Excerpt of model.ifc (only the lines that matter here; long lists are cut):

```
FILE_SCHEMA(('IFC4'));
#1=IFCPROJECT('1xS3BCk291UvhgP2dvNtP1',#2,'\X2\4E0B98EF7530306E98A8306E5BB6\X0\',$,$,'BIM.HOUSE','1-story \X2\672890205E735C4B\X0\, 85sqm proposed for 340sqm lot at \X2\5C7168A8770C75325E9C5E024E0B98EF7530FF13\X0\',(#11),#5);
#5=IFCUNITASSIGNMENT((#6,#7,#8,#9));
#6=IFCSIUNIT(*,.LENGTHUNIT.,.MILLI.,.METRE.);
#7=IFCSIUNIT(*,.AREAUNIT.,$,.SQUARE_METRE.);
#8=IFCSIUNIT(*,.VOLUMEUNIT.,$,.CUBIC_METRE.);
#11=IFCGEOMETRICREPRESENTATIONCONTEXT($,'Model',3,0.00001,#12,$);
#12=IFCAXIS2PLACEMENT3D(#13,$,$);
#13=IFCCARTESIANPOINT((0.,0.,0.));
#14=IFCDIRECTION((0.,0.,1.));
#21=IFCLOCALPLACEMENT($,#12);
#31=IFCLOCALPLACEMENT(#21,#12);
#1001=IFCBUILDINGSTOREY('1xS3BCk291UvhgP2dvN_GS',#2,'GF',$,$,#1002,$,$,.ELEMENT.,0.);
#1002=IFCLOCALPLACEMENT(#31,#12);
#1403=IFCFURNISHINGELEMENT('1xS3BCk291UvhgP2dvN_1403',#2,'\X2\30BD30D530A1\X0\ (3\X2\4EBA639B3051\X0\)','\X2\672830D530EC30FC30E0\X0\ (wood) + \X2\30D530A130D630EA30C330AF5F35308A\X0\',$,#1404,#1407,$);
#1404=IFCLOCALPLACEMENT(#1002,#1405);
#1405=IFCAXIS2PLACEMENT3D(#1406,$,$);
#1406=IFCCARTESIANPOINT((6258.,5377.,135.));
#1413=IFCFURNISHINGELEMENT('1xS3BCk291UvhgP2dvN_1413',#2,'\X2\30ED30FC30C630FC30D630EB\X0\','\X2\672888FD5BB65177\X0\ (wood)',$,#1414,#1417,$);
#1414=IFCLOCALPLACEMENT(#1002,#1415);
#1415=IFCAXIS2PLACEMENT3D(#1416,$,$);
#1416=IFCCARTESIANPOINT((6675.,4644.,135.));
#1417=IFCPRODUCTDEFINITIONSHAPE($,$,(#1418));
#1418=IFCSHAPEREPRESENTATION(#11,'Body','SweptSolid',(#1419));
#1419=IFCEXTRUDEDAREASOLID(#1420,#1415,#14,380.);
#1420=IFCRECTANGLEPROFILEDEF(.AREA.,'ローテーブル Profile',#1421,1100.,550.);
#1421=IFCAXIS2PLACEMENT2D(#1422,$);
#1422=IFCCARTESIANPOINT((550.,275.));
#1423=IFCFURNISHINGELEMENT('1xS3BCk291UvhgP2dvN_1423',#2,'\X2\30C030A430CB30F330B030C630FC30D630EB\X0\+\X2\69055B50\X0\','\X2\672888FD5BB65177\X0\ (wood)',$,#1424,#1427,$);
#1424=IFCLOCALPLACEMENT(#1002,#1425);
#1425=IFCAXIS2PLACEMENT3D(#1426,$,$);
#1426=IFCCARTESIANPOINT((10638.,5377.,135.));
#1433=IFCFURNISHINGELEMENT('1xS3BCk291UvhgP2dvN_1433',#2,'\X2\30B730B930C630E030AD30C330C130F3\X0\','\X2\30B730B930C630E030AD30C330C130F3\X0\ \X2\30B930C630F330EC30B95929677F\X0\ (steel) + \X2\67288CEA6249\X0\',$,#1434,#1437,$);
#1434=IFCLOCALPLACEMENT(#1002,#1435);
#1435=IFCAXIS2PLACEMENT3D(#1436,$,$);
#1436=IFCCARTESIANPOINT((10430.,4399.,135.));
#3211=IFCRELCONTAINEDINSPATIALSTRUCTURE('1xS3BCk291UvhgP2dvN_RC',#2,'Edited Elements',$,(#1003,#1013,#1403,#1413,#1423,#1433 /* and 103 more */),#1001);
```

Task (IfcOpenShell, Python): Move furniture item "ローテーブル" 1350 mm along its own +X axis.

```python
import ifcopenshell
import ifcopenshell.api.geometry
import ifcopenshell.util.placement
import ifcopenshell.util.unit

model = ifcopenshell.open("model.ifc")
unit_scale = ifcopenshell.util.unit.calculate_unit_scale(model)

item = model.by_guid("1xS3BCk291UvhgP2dvN_1413")
matrix = ifcopenshell.util.placement.get_local_placement(item.ObjectPlacement)
matrix[:3, 3] += matrix[:3, 0] * 1.35 / unit_scale
ifcopenshell.api.geometry.edit_object_placement(model, product=item, matrix=matrix, is_si=False)

print(ifcopenshell.util.placement.get_local_placement(item.ObjectPlacement).round(3) + 0.0)

model.write("model-out.ifc")
```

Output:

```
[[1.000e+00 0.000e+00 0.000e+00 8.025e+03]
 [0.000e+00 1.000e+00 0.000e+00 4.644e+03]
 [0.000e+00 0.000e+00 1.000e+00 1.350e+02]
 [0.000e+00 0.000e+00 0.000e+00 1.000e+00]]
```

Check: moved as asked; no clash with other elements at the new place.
